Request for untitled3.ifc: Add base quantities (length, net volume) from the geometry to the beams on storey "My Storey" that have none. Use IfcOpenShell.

First a look at what the model holds.

```python
import ifcopenshell
import ifcopenshell.util.element
import ifcopenshell.util.unit

model = ifcopenshell.open("untitled3.ifc")
print(model.schema)
for unit_type in ("LENGTHUNIT", "AREAUNIT", "VOLUMEUNIT"):
    print(unit_type, ifcopenshell.util.unit.calculate_unit_scale(model, unit_type))
storey = next(s for s in model.by_type("IfcBuildingStorey") if s.Name == "My Storey")
beams = [e for e in ifcopenshell.util.element.get_decomposition(storey) if e.is_a("IfcBeam")]
for e in sorted(beams, key=lambda e: e.id()):
    print(e.id(), e.is_a(), e.Name, list(ifcopenshell.util.element.get_psets(e, qtos_only=True)), sep=" | ")
```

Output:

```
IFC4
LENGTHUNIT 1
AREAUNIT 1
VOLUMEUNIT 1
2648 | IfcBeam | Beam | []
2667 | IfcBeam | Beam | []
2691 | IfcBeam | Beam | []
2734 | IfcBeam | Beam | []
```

```python
import ifcopenshell
import ifcopenshell.api.pset
import ifcopenshell.geom
import ifcopenshell.util.element
import ifcopenshell.util.shape
import ifcopenshell.util.unit

model = ifcopenshell.open("untitled3.ifc")
unit_scale = ifcopenshell.util.unit.calculate_unit_scale(model)
volume_scale = ifcopenshell.util.unit.calculate_unit_scale(model, "VOLUMEUNIT")
settings = ifcopenshell.geom.settings()

storey = next(s for s in model.by_type("IfcBuildingStorey") if s.Name == "My Storey")
beams = [e for e in ifcopenshell.util.element.get_decomposition(storey) if e.is_a("IfcBeam")]

for e in sorted(beams, key=lambda e: e.id()):
    if ifcopenshell.util.element.get_psets(e, qtos_only=True, should_inherit=False):
        continue
    # Geometry comes back in metres, in the element's own axes.
    shape = ifcopenshell.geom.create_shape(settings, e)
    values = {
        "Length": ifcopenshell.util.shape.get_max_xyz(shape.geometry) / unit_scale,
        "NetVolume": ifcopenshell.util.shape.get_volume(shape.geometry) / volume_scale,
    }
    qto = ifcopenshell.api.pset.add_qto(model, product=e, name="Qto_BeamBaseQuantities")
    ifcopenshell.api.pset.edit_qto(model, qto=qto, properties=values)
    print(e.id(), {k: round(v, 3) for k, v in values.items()})

model.write("untitled3_v2.ifc")
```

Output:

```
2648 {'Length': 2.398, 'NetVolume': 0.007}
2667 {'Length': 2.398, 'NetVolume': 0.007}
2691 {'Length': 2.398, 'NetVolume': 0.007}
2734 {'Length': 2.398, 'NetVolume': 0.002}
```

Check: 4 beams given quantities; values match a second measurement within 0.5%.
